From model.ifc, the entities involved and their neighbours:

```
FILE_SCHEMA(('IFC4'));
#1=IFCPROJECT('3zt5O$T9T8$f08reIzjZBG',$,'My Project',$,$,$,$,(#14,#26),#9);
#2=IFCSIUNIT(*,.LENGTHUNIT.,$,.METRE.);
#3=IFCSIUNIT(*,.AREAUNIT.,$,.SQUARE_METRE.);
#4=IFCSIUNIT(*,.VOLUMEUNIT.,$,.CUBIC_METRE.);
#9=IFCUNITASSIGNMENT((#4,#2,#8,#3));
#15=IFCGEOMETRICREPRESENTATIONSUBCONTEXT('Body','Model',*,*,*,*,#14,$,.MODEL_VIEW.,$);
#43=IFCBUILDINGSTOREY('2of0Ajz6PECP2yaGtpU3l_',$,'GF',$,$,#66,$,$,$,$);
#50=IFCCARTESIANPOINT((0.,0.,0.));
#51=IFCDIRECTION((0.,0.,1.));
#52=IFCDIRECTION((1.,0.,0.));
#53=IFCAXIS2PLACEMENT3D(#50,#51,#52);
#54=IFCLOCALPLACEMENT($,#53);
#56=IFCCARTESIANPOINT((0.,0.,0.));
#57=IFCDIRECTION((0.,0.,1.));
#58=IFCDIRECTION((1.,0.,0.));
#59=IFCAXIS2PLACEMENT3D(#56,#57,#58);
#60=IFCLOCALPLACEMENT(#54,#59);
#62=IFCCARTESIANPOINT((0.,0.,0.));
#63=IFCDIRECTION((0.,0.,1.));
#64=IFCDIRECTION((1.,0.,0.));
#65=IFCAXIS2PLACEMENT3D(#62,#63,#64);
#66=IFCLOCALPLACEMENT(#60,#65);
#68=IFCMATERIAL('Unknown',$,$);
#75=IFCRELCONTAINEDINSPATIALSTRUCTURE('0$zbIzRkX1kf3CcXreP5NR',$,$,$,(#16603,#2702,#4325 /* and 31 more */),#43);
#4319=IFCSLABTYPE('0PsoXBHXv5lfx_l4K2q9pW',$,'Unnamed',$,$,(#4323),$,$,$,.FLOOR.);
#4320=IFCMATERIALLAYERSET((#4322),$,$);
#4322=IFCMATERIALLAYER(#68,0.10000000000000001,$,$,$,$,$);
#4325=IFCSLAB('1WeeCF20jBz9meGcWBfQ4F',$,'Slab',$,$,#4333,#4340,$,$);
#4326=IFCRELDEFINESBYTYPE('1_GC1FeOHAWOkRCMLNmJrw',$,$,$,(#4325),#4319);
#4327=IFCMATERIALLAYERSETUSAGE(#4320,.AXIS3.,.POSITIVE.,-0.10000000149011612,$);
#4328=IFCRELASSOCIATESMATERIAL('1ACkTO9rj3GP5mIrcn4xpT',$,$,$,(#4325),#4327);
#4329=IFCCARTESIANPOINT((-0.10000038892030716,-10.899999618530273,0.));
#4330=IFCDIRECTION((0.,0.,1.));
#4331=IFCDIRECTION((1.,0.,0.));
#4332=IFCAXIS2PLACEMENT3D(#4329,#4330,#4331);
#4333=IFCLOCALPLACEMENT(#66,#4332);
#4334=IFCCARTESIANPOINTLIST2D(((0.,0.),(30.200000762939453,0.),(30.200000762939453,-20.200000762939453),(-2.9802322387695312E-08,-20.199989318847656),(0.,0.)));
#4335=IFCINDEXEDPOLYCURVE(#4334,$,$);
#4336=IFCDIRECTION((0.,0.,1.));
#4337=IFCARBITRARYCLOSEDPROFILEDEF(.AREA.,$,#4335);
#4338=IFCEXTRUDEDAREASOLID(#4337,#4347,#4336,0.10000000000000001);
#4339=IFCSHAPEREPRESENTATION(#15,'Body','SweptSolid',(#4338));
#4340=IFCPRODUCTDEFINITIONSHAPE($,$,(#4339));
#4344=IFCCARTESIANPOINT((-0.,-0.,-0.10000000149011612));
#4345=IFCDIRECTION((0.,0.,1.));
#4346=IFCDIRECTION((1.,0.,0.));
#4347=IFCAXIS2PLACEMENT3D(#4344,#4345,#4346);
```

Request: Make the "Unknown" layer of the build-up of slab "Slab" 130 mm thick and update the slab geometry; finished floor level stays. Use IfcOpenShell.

```python
import ifcopenshell
import ifcopenshell.util.element
import ifcopenshell.util.representation

model = ifcopenshell.open("model.ifc")

layer_set = model.by_id(4320)
layer = next(l for l in layer_set.MaterialLayers if l.Material and l.Material.Name == "Unknown")
change = 0.13 - layer.LayerThickness
layer.LayerThickness += change

# Geometry does not follow the layer set by itself.
slabs = [e for e in ifcopenshell.util.element.get_elements_by_material(model, layer_set) if e.is_a("IfcSlab")]
for slab in sorted(slabs, key=lambda e: e.id()):
    body = ifcopenshell.util.representation.get_representation(slab, "Model", "Body")
    solid = body.Items[0]
    old_depth = solid.Depth
    solid.Depth += change
    # Extruded upwards: lower the start of the extrusion so the top stays.
    x, y, z = solid.Position.Location.Coordinates
    solid.Position.Location = model.createIfcCartesianPoint((x, y, z - change))
    print(slab.id(), f"{old_depth:g} -> {solid.Depth:g}")

# The layers are counted up from the underside, which has moved.
for usage in {ifcopenshell.util.element.get_material(slab) for slab in slabs}:
    usage.OffsetFromReferenceLine -= change

model.write("model_edited.ifc")
```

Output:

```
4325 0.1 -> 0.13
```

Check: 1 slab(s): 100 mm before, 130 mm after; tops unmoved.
